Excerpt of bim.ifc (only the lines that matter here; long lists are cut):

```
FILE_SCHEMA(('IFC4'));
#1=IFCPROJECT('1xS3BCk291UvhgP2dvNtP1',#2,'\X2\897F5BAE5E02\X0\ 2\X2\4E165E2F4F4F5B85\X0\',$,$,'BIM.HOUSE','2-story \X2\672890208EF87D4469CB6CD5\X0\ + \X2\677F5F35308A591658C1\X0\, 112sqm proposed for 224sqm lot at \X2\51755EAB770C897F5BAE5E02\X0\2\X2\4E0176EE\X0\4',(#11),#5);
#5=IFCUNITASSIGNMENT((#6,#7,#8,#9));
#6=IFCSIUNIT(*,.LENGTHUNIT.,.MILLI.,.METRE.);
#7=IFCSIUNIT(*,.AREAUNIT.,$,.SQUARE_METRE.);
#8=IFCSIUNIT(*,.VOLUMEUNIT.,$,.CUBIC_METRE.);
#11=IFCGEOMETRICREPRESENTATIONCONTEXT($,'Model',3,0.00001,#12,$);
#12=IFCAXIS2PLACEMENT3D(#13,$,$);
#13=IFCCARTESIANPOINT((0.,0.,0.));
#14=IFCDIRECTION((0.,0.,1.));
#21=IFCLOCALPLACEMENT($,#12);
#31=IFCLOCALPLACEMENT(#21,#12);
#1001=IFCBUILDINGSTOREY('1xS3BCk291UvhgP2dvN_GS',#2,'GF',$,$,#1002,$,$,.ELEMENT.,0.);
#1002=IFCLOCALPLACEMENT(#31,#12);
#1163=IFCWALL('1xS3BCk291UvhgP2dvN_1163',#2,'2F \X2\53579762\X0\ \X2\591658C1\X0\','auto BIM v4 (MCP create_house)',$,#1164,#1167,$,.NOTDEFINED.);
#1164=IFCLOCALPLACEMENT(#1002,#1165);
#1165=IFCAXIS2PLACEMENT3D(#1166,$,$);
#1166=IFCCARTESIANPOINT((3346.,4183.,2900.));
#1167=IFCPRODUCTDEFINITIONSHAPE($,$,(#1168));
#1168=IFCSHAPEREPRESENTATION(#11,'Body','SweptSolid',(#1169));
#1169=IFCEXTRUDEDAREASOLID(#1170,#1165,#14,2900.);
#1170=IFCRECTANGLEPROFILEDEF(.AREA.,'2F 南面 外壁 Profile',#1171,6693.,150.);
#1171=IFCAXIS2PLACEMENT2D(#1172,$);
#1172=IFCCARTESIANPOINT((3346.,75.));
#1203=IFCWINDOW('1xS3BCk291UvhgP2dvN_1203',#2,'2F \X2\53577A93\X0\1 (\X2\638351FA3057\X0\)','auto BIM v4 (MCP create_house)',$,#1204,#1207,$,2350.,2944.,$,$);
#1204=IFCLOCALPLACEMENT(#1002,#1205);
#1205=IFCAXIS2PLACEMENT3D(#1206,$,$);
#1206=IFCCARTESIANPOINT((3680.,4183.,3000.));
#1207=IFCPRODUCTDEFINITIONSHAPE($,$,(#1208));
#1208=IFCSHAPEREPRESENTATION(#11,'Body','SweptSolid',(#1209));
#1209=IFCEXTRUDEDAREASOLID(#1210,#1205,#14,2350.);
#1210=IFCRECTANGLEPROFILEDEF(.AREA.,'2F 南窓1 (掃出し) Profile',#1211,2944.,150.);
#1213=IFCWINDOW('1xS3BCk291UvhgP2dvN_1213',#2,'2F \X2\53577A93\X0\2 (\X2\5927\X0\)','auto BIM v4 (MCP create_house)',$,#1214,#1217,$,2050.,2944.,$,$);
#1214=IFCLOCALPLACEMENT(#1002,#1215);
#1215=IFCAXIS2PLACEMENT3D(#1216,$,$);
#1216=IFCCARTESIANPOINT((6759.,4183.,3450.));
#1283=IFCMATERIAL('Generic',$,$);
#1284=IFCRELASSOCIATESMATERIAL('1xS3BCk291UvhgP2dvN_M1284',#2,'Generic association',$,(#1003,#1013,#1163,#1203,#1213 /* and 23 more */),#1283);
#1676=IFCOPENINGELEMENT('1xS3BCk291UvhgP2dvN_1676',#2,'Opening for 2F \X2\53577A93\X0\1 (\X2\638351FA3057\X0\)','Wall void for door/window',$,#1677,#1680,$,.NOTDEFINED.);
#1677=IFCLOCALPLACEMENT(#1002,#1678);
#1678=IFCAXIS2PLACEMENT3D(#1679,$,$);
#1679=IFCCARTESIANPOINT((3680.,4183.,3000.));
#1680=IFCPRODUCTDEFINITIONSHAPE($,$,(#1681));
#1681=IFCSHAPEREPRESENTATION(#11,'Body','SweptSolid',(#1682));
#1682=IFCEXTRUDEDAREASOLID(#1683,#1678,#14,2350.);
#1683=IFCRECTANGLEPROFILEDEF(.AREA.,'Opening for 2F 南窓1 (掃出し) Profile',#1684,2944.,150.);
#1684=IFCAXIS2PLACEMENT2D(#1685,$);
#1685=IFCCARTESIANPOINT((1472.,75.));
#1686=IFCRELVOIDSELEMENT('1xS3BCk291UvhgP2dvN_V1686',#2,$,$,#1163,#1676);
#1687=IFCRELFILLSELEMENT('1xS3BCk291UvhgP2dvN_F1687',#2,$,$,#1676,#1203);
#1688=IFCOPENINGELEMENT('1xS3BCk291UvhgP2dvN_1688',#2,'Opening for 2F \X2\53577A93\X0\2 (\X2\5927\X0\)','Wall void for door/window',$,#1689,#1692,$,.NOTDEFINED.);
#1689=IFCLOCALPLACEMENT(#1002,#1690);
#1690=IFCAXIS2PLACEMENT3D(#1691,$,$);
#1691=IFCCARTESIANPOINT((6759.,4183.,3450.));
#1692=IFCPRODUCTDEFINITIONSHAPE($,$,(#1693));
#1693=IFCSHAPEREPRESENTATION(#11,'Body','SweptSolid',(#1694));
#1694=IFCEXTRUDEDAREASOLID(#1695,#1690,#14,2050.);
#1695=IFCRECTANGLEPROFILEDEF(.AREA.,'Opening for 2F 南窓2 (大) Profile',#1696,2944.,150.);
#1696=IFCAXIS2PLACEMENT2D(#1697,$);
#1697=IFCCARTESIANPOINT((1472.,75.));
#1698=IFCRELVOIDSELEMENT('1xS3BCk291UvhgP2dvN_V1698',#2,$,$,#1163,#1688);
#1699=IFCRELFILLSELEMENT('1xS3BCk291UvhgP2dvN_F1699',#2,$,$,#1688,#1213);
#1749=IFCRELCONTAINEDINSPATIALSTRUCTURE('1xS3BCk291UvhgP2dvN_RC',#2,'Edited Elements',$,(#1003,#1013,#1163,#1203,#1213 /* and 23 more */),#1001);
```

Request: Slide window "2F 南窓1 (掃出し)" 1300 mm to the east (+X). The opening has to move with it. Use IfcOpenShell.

```python
import ifcopenshell
import ifcopenshell.api.geometry
import ifcopenshell.util.placement
import ifcopenshell.util.unit

model = ifcopenshell.open("bim.ifc")
unit_scale = ifcopenshell.util.unit.calculate_unit_scale(model)

window = model.by_id(1203)
opening = window.FillsVoids[0].RelatingOpeningElement
wall = opening.VoidsElements[0].RelatingBuildingElement

wall_matrix = ifcopenshell.util.placement.get_local_placement(wall.ObjectPlacement)
shift = wall_matrix[:3, 0] * 1.3 / unit_scale
before = ifcopenshell.util.placement.get_local_placement(window.ObjectPlacement)[:3, 3].copy()

# The window is not placed relative to its opening, so move both.
for product in (opening, window):
    matrix = ifcopenshell.util.placement.get_local_placement(product.ObjectPlacement)
    matrix[:3, 3] += shift
    ifcopenshell.api.geometry.edit_object_placement(model, product=product, matrix=matrix, is_si=False)

after = ifcopenshell.util.placement.get_local_placement(window.ObjectPlacement)[:3, 3]
print("window moved by", (after - before).round(3) + 0.0)

model.write("bim_v2.ifc")
```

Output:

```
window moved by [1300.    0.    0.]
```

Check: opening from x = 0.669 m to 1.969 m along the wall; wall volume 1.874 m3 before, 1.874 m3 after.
